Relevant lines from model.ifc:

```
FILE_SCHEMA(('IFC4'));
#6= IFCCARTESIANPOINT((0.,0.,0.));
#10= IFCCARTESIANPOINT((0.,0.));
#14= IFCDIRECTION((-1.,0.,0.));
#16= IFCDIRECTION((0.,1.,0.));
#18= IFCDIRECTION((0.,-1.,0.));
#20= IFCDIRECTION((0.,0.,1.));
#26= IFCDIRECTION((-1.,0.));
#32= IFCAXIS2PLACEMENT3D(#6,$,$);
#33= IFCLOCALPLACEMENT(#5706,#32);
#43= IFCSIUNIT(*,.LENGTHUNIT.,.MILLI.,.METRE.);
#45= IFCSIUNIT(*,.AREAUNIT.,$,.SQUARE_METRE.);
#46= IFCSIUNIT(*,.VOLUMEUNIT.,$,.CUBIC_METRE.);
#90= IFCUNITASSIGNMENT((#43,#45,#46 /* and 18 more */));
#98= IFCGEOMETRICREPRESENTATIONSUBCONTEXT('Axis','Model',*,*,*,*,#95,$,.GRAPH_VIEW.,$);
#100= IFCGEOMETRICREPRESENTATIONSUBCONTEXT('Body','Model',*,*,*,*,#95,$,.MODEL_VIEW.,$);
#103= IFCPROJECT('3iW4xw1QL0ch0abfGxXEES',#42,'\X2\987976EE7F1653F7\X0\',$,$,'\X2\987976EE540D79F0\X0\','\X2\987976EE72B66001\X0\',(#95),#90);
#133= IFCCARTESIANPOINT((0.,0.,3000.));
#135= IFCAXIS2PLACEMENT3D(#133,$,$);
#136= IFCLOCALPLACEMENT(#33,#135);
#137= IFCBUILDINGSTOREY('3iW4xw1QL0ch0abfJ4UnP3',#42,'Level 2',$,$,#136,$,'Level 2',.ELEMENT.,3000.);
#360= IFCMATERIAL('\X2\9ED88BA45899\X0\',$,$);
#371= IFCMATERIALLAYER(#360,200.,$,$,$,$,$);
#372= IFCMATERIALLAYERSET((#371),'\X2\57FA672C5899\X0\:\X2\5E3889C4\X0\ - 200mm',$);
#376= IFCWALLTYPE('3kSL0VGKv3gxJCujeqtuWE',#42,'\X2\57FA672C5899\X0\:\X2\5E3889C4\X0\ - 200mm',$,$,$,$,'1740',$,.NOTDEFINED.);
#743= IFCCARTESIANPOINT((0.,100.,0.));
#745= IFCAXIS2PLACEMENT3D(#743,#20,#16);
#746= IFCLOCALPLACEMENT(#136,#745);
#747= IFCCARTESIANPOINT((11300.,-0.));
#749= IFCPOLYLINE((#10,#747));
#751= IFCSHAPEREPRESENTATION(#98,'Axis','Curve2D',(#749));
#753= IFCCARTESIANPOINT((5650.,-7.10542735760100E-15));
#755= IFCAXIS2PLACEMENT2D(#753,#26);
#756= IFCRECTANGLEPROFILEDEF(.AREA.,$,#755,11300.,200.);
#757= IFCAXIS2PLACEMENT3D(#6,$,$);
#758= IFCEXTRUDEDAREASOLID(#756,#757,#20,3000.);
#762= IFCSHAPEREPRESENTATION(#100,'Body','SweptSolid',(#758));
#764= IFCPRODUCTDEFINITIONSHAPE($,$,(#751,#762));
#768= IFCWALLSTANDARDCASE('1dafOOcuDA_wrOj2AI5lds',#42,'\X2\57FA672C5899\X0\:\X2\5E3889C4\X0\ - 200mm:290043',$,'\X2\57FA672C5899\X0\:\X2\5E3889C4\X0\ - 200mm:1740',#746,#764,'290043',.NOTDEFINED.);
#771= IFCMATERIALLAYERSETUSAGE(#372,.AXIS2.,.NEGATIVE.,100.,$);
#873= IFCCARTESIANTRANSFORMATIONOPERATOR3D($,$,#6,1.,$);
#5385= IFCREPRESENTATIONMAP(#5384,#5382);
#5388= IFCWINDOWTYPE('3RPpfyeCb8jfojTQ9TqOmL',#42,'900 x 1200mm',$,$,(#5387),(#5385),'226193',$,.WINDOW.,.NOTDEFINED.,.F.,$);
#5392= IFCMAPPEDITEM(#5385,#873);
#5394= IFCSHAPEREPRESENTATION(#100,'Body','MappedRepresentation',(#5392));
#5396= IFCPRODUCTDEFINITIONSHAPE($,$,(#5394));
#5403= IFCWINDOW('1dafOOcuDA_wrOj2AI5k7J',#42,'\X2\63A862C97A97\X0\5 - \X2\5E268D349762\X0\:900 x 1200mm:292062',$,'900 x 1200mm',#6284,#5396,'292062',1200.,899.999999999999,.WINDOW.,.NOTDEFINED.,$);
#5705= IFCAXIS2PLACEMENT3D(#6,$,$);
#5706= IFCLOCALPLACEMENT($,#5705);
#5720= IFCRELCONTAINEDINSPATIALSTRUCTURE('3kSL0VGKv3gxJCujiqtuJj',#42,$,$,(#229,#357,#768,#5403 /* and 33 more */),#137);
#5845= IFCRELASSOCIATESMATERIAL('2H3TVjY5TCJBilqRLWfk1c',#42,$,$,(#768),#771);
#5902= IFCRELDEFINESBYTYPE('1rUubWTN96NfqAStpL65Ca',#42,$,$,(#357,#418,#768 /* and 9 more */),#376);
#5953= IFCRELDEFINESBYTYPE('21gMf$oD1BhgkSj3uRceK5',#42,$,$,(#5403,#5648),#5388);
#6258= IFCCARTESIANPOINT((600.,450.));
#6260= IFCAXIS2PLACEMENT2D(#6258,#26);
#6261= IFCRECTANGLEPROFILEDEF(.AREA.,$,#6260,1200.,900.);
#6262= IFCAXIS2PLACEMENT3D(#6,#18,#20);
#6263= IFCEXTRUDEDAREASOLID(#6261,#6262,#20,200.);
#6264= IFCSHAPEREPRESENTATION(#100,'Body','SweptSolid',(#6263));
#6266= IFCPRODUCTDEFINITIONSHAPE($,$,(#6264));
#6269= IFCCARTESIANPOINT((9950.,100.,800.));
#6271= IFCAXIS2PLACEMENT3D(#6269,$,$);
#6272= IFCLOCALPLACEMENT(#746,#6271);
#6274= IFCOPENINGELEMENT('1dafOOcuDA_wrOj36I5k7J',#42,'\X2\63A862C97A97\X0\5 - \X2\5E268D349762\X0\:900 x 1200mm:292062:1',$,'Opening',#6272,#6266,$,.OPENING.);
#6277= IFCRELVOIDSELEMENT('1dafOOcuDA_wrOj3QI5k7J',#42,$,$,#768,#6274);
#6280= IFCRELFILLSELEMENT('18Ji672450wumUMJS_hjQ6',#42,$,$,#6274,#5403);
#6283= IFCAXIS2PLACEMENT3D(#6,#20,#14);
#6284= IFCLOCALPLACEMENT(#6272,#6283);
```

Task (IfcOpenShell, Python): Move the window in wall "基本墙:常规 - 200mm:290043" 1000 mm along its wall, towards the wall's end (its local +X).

```python
import ifcopenshell
import ifcopenshell.api.geometry
import ifcopenshell.util.placement

model = ifcopenshell.open("model.ifc")

window = model.by_guid("1dafOOcuDA_wrOj2AI5k7J")
opening = window.FillsVoids[0].RelatingOpeningElement
wall = opening.VoidsElements[0].RelatingBuildingElement

wall_matrix = ifcopenshell.util.placement.get_local_placement(wall.ObjectPlacement)
shift = wall_matrix[:3, 0] * 1000.0
before = ifcopenshell.util.placement.get_local_placement(window.ObjectPlacement)[:3, 3].copy()

# The window is placed relative to its opening, so it follows when the opening moves.
matrix = ifcopenshell.util.placement.get_local_placement(opening.ObjectPlacement)
matrix[:3, 3] += shift
ifcopenshell.api.geometry.edit_object_placement(
    model, product=opening, matrix=matrix, is_si=False, should_transform_children=True
)

after = ifcopenshell.util.placement.get_local_placement(window.ObjectPlacement)[:3, 3]
print("window moved by", (after - before).round(3) + 0.0)

model.write("model_updated.ifc")
```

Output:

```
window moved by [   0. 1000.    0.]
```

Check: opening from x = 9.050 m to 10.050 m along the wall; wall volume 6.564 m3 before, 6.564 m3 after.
